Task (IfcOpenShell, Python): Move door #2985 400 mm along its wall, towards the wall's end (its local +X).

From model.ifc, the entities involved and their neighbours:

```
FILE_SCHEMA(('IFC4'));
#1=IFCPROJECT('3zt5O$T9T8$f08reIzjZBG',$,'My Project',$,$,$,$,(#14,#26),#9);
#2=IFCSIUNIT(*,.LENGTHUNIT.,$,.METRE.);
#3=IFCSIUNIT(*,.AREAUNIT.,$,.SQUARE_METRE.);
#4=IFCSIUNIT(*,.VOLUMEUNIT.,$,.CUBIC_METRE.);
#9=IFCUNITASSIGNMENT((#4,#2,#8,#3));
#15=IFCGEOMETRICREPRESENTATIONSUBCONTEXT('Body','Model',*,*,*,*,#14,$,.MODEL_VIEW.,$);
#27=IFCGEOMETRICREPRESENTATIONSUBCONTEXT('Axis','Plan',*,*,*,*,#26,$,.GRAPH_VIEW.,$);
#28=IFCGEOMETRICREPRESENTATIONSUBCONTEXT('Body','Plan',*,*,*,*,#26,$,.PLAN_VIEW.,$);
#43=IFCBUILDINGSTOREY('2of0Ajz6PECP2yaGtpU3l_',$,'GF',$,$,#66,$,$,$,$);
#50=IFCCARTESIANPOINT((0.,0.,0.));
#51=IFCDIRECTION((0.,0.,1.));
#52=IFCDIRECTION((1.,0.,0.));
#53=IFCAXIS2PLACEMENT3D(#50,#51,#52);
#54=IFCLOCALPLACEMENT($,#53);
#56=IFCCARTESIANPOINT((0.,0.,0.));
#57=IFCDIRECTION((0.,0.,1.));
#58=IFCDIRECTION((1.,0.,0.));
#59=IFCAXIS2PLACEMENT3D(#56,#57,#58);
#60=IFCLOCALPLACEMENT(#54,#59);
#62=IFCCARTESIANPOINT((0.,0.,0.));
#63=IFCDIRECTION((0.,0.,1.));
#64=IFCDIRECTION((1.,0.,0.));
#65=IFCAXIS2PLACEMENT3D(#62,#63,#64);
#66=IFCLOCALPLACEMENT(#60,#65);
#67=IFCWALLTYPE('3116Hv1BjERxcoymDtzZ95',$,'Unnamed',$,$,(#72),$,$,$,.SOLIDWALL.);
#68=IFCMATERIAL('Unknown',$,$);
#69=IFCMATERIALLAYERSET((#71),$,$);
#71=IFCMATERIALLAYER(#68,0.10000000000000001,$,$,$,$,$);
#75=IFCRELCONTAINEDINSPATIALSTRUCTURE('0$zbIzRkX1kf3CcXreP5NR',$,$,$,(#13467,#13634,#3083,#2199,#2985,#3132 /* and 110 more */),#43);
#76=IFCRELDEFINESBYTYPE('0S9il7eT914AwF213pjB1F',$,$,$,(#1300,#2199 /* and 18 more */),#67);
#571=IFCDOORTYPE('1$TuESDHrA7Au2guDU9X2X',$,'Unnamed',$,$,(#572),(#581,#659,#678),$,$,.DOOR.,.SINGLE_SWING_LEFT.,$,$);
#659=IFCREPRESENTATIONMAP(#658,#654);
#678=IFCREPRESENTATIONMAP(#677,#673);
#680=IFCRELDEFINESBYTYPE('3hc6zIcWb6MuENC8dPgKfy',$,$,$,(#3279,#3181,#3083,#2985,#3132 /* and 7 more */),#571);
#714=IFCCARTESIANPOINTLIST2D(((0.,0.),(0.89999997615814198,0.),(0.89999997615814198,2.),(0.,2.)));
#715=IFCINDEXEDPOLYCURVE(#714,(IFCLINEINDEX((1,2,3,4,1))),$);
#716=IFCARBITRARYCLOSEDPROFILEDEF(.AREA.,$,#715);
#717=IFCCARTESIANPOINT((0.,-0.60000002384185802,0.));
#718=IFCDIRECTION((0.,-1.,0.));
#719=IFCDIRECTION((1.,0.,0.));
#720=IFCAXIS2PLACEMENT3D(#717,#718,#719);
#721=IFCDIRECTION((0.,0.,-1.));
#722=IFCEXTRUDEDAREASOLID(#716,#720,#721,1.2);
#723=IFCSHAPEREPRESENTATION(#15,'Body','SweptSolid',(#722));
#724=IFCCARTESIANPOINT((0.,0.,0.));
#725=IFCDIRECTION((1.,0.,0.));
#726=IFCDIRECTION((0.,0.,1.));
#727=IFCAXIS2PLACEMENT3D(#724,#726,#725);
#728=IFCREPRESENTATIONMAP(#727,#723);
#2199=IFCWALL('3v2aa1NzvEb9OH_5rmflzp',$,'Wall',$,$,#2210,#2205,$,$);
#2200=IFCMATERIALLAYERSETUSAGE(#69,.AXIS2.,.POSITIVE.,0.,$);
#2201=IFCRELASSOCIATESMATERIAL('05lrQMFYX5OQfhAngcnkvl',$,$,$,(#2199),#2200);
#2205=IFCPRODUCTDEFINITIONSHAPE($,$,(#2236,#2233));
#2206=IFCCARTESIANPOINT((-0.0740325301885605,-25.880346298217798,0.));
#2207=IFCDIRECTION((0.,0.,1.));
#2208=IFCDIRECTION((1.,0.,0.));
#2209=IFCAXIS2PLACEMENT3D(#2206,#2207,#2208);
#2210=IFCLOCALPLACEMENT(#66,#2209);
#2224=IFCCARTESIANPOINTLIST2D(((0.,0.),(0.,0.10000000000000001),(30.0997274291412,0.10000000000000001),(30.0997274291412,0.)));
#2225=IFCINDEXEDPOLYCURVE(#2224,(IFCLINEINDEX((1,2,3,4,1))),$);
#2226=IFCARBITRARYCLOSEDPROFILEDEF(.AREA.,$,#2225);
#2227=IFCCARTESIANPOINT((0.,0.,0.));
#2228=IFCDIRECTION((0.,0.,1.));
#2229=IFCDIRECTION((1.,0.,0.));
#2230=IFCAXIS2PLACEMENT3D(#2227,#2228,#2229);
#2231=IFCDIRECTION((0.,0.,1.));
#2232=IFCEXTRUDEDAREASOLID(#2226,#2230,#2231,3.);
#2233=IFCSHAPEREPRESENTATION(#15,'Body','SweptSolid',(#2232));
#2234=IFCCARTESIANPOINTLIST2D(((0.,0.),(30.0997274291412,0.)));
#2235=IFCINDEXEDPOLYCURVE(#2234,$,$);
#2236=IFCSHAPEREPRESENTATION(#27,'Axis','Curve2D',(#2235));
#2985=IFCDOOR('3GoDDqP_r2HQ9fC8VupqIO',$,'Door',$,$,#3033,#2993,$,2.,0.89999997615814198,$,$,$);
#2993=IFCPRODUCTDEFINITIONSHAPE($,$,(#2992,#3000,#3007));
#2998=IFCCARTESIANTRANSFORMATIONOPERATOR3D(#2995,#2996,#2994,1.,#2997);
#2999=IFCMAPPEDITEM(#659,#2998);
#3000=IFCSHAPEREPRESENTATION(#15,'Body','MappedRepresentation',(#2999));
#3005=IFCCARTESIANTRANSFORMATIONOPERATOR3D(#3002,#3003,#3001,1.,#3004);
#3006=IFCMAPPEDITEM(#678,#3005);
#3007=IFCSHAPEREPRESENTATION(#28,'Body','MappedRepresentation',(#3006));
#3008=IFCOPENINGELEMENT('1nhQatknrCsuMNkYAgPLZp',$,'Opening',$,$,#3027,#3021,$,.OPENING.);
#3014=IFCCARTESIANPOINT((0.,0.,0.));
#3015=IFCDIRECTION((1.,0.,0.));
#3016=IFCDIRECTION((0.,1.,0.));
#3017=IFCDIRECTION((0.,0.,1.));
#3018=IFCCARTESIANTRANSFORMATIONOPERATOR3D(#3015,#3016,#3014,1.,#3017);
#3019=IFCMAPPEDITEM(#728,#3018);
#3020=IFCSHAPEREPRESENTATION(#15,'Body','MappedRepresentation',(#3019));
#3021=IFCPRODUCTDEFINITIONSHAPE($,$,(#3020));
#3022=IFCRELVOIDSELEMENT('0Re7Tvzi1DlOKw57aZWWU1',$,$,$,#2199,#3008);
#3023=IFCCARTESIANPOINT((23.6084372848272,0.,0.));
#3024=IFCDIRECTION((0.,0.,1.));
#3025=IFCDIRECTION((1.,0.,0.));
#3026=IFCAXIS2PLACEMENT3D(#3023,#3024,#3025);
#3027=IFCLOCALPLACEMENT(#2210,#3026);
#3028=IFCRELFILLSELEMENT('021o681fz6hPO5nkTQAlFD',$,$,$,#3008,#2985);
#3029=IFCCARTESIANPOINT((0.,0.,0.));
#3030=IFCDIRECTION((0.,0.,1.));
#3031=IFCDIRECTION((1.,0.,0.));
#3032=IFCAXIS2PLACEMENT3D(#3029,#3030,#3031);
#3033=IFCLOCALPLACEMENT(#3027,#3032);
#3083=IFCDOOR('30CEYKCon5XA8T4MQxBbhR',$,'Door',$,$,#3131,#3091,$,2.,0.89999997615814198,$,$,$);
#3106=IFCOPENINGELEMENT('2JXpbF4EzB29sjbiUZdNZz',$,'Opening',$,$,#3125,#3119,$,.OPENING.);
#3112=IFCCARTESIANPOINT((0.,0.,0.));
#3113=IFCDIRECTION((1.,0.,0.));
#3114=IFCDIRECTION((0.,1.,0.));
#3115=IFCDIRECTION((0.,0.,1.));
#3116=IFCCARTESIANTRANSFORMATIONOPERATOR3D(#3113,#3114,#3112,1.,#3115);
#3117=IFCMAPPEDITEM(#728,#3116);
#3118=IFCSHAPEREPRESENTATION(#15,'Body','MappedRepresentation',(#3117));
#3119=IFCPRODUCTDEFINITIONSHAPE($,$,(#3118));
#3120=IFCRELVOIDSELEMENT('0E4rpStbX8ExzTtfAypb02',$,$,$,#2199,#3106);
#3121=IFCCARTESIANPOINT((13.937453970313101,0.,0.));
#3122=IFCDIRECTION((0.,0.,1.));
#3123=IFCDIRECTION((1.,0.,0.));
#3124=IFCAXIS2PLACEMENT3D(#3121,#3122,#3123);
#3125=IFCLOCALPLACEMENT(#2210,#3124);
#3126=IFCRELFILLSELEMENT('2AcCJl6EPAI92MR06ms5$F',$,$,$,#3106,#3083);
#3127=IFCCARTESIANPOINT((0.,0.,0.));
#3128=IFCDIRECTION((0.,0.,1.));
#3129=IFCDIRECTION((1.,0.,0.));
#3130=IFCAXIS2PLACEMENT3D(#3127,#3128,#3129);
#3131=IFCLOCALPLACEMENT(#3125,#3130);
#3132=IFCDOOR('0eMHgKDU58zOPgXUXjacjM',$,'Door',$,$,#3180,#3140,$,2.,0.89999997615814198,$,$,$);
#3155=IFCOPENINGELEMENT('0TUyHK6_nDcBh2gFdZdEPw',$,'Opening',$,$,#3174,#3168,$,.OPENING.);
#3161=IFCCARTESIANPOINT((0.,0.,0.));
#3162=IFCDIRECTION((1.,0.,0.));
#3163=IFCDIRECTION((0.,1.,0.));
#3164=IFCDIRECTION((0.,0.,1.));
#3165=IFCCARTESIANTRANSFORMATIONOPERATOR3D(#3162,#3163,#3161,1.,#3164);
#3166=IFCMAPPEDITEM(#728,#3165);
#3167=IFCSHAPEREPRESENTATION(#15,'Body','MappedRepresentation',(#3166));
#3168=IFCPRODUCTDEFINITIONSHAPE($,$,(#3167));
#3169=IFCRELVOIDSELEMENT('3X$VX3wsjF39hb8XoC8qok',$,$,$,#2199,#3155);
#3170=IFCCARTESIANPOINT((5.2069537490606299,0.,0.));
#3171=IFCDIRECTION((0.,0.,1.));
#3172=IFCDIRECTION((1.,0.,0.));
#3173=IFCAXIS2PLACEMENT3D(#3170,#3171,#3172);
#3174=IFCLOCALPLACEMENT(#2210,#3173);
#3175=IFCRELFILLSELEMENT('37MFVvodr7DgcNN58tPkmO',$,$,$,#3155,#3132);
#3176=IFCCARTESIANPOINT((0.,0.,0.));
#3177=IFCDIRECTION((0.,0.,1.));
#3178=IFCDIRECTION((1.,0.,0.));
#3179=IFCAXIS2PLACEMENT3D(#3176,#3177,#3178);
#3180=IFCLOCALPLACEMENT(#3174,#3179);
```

```python
import ifcopenshell
import ifcopenshell.api.geometry
import ifcopenshell.util.placement
import ifcopenshell.util.unit

model = ifcopenshell.open("model.ifc")
unit_scale = ifcopenshell.util.unit.calculate_unit_scale(model)

door = model.by_guid("3GoDDqP_r2HQ9fC8VupqIO")
opening = door.FillsVoids[0].RelatingOpeningElement
wall = opening.VoidsElements[0].RelatingBuildingElement

wall_matrix = ifcopenshell.util.placement.get_local_placement(wall.ObjectPlacement)
shift = wall_matrix[:3, 0] * 0.4 / unit_scale
before = ifcopenshell.util.placement.get_local_placement(door.ObjectPlacement)[:3, 3].copy()

# The door is placed relative to its opening, so it follows when the opening moves.
matrix = ifcopenshell.util.placement.get_local_placement(opening.ObjectPlacement)
matrix[:3, 3] += shift
ifcopenshell.api.geometry.edit_object_placement(
    model, product=opening, matrix=matrix, is_si=False, should_transform_children=True
)

after = ifcopenshell.util.placement.get_local_placement(door.ObjectPlacement)[:3, 3]
print("door moved by", (after - before).round(3) + 0.0)

model.write("model-out.ifc")
```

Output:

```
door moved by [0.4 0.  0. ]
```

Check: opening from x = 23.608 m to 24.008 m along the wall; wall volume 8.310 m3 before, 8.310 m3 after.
